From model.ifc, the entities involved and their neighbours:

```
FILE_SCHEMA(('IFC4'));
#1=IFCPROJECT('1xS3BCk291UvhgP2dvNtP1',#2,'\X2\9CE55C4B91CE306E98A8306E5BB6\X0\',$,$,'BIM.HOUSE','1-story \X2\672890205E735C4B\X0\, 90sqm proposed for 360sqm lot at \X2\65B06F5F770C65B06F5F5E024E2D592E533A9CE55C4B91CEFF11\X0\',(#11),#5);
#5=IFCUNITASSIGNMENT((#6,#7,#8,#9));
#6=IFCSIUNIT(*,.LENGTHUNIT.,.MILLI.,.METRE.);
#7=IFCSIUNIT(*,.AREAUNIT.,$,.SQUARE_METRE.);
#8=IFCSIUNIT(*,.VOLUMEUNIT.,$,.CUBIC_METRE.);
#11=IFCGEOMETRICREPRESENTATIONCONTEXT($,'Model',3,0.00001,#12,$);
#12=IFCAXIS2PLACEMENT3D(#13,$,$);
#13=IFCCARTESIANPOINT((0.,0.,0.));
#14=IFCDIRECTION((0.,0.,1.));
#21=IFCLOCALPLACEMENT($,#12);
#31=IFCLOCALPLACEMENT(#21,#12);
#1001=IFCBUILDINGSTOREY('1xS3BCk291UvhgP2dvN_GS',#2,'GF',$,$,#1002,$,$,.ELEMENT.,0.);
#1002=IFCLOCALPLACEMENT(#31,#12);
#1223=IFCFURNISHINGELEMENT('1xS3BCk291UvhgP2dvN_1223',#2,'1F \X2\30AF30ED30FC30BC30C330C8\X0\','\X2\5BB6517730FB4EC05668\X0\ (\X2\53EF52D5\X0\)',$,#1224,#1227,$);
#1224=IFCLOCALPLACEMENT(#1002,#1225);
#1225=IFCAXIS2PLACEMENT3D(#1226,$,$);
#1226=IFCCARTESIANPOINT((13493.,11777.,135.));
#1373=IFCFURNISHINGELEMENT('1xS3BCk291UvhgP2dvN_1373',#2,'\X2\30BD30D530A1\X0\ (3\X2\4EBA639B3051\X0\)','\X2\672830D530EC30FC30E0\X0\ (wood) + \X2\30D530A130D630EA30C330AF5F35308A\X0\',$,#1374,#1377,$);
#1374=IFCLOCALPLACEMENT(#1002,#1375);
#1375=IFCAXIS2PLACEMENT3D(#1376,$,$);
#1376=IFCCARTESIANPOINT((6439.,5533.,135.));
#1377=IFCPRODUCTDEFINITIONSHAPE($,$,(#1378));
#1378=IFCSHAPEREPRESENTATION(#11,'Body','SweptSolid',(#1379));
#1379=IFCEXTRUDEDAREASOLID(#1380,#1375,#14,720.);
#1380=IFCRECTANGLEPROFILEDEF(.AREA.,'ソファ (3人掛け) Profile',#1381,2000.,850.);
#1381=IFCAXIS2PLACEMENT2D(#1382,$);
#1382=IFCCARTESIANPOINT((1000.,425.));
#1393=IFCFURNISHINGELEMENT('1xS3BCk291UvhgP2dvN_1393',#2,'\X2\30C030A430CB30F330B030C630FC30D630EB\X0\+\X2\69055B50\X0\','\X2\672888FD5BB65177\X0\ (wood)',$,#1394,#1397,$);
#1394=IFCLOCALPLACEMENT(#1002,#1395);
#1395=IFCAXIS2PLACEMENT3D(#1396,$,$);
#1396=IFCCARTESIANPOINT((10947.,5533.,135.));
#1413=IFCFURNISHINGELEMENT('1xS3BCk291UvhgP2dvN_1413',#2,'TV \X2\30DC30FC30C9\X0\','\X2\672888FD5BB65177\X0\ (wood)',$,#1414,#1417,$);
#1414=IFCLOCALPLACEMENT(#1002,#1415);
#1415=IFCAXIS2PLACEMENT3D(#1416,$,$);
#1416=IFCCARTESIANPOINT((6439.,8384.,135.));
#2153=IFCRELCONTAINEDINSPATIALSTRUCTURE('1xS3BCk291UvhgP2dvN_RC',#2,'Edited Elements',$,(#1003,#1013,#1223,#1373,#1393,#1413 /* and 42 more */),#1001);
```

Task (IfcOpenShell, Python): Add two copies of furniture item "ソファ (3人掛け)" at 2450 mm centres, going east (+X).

```python
import numpy as np
import ifcopenshell
import ifcopenshell.api.geometry
import ifcopenshell.api.root
import ifcopenshell.util.element
import ifcopenshell.util.placement

model = ifcopenshell.open("model.ifc")


def reuse_history(source, copy):
    """copy_class also copies each property set's owner history, people and application; keep the originals."""
    for rel in copy.IsDefinedBy:
        if rel.is_a("IfcRelDefinesByProperties") and (history := rel.RelatingPropertyDefinition.OwnerHistory):
            rel.RelatingPropertyDefinition.OwnerHistory = source.OwnerHistory
            ifcopenshell.util.element.remove_deep2(model, history)


source = model.by_guid("1xS3BCk291UvhgP2dvN_1373")
base = ifcopenshell.util.placement.get_local_placement(source.ObjectPlacement)
step = np.array([1.0, 0.0, 0.0]) * 2450.0

for i in range(1, 3):
    copy = ifcopenshell.api.root.copy_class(model, product=source)
    copy.Representation = ifcopenshell.util.element.copy_deep(
        model, source.Representation, exclude=["IfcGeometricRepresentationContext", "IfcRepresentationMap"]
    )
    reuse_history(source, copy)
    matrix = base.copy()
    matrix[:3, 3] += i * step
    print("added at", matrix[:3, 3].round(3) + 0.0)
    ifcopenshell.api.geometry.edit_object_placement(model, product=copy, matrix=matrix, is_si=False)

model.write("model_edited.ifc")
```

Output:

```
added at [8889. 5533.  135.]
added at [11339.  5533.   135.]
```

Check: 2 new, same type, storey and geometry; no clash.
